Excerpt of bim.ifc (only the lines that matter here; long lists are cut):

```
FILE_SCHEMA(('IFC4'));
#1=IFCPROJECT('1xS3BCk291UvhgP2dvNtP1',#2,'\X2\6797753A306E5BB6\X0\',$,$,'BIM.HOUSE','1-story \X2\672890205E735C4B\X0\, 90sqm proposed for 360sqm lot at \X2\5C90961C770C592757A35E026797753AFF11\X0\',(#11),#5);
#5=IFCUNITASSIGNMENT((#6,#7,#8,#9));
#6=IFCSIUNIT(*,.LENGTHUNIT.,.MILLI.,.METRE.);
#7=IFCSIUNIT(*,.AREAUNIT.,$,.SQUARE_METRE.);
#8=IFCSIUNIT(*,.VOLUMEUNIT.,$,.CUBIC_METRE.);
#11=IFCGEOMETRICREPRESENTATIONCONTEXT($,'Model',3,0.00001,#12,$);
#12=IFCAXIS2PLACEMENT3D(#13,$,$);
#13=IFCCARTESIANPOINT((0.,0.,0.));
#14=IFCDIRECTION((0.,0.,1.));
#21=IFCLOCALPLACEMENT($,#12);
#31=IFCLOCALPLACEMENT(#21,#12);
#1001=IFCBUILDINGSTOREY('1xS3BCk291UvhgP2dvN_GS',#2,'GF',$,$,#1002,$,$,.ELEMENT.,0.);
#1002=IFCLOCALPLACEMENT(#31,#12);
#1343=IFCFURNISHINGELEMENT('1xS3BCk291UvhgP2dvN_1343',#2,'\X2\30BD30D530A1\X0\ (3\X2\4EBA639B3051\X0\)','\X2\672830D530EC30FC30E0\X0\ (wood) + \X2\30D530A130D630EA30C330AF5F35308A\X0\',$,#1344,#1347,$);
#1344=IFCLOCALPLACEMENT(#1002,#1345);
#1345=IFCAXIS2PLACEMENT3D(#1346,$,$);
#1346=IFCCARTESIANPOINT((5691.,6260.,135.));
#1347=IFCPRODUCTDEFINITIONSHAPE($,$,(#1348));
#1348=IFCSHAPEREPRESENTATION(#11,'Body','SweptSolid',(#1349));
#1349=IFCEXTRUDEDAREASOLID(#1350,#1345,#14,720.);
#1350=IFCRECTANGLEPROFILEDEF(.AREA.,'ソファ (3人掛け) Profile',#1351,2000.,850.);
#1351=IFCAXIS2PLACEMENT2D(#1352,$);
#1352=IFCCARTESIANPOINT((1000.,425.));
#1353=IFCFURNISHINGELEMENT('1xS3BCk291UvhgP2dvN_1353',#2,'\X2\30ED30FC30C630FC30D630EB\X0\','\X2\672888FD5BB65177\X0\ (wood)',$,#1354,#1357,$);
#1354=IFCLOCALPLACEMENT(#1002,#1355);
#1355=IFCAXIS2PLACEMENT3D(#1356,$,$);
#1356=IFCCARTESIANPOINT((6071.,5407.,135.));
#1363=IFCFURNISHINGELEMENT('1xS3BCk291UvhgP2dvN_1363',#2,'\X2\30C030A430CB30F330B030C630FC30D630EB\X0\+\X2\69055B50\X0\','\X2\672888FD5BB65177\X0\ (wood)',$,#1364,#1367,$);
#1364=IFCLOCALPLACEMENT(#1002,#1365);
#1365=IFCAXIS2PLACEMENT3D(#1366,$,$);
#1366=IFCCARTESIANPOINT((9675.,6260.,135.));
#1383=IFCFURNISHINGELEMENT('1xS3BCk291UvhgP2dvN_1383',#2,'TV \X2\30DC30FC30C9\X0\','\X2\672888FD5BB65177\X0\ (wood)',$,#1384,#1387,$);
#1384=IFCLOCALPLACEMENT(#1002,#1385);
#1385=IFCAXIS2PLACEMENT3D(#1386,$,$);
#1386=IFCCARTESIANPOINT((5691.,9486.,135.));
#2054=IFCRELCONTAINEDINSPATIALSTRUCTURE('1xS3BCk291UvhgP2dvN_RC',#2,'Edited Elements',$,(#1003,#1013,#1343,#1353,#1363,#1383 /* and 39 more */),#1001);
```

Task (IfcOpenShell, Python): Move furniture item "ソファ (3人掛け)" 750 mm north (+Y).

```python
import ifcopenshell
import ifcopenshell.api.geometry
import ifcopenshell.util.placement

model = ifcopenshell.open("bim.ifc")

item = model.by_guid("1xS3BCk291UvhgP2dvN_1343")
matrix = ifcopenshell.util.placement.get_local_placement(item.ObjectPlacement)
matrix[1, 3] += 750.0
ifcopenshell.api.geometry.edit_object_placement(model, product=item, matrix=matrix, is_si=False)

print(ifcopenshell.util.placement.get_local_placement(item.ObjectPlacement).round(3) + 0.0)

model.write("bim_edited.ifc")
```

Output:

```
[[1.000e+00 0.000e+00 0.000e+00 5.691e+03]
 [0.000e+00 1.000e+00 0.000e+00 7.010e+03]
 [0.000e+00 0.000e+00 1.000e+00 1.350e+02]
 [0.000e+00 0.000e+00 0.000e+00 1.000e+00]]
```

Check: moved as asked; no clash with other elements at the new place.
